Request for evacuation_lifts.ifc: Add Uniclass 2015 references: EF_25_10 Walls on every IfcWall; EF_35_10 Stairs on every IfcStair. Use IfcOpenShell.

First a look at what the model holds.

```python
import ifcopenshell

model = ifcopenshell.open("evacuation_lifts.ifc")
print(model.schema)
print("classifications:", [c.Name for c in model.by_type("IfcClassification")])
for ifc_class in ("IfcDoor", "IfcRoof", "IfcStair", "IfcWall", "IfcWindow"):
    print(ifc_class, len(model.by_type(ifc_class)))
```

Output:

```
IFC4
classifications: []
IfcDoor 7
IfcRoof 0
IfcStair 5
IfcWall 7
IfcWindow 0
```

```python
import ifcopenshell
import ifcopenshell.api.classification

model = ifcopenshell.open("evacuation_lifts.ifc")

system = ifcopenshell.api.classification.add_classification(model, classification="Uniclass 2015")

codes = {
    "IfcWall": ("EF_25_10", "Walls"),
    "IfcStair": ("EF_35_10", "Stairs"),
}
for ifc_class, (code, name) in codes.items():
    products = model.by_type(ifc_class)
    ifcopenshell.api.classification.add_reference(
        model, products=products, classification=system, identification=code, name=name
    )
    print(code, len(products))

model.write("evacuation_lifts_rev.ifc")
```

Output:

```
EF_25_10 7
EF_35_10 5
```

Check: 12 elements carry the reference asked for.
